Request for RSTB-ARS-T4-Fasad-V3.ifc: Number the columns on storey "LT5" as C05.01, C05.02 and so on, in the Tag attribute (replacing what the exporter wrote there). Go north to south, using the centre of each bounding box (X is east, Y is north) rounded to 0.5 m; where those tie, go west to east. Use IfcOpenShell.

First a look at what the model holds.

```python
import ifcopenshell
import ifcopenshell.util.element
import ifcopenshell.util.placement

model = ifcopenshell.open("RSTB-ARS-T4-Fasad-V3.ifc")
print(model.schema)
storey = next(s for s in model.by_type("IfcBuildingStorey") if s.Name == "LT5")
columns = [e for e in ifcopenshell.util.element.get_decomposition(storey) if e.is_a("IfcColumn")]
for e in sorted(columns, key=lambda e: e.id()):
    origin = ifcopenshell.util.placement.get_local_placement(e.ObjectPlacement)[:3, 3]
    print(e.id(), e.Tag, e.Name, origin.round(2) + 0.0, sep=" | ")
```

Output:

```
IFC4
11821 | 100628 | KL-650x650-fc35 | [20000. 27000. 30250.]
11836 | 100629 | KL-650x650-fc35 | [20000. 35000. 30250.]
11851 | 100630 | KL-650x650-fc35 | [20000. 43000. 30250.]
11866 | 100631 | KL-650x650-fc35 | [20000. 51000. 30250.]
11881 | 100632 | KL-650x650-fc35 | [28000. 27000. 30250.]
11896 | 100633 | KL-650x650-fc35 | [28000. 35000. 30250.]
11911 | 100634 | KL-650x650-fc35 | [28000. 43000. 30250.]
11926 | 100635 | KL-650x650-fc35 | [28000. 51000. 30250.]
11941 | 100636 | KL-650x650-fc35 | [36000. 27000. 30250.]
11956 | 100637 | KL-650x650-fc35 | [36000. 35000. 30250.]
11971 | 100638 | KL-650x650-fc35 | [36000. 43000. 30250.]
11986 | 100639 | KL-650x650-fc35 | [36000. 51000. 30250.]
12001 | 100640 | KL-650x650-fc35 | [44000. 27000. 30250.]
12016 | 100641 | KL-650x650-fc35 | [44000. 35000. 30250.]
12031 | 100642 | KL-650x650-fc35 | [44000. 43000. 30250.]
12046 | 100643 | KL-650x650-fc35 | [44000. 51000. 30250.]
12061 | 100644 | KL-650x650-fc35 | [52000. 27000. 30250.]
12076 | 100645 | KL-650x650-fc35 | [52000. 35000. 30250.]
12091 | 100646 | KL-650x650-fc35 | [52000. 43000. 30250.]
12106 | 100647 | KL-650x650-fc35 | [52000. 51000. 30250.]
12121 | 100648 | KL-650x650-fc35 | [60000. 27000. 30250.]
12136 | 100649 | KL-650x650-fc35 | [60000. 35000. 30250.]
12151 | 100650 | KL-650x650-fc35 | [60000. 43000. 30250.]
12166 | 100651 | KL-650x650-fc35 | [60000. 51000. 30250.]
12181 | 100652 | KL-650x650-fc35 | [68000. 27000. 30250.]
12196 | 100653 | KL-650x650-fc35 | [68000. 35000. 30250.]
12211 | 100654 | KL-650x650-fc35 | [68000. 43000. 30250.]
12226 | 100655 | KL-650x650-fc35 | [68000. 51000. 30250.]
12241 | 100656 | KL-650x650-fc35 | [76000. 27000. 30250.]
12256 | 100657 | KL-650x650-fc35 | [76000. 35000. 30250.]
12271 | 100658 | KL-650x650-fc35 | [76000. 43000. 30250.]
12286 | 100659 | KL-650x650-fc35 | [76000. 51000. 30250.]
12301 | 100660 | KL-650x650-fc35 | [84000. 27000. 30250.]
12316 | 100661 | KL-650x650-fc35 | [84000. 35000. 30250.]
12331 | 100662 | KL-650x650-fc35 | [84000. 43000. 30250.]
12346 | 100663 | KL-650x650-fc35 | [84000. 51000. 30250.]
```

```python
import ifcopenshell
import ifcopenshell.geom
import ifcopenshell.util.element
import ifcopenshell.util.shape

model = ifcopenshell.open("RSTB-ARS-T4-Fasad-V3.ifc")
settings = ifcopenshell.geom.settings()
settings.set("use-world-coords", True)


def centre(element):
    shape = ifcopenshell.geom.create_shape(settings, element)
    return ifcopenshell.util.shape.get_bbox_centroid(shape.geometry)


storey = next(s for s in model.by_type("IfcBuildingStorey") if s.Name == "LT5")
columns = [e for e in ifcopenshell.util.element.get_decomposition(storey) if e.is_a("IfcColumn")]

# Insertion points can sit at a corner or the storey origin, so sort by the geometry (in metres).
centres = {e: centre(e) for e in columns}
columns.sort(key=lambda e: (-round(centres[e][1] / 0.5), centres[e][0]))

for i, e in enumerate(columns, start=1):
    number = f"C05.{i:02d}"
    e.Tag = number
    print(e.id(), number)

model.write("RSTB-ARS-T4-Fasad-V3_edited.ifc")
```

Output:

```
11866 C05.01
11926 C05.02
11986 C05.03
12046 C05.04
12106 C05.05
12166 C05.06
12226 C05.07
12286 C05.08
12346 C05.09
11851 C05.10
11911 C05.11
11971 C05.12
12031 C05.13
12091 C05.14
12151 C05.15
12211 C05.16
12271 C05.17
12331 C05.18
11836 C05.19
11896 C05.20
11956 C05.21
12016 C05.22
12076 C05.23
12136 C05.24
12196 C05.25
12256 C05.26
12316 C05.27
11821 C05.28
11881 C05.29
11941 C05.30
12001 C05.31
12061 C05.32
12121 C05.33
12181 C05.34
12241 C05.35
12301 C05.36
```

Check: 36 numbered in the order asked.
